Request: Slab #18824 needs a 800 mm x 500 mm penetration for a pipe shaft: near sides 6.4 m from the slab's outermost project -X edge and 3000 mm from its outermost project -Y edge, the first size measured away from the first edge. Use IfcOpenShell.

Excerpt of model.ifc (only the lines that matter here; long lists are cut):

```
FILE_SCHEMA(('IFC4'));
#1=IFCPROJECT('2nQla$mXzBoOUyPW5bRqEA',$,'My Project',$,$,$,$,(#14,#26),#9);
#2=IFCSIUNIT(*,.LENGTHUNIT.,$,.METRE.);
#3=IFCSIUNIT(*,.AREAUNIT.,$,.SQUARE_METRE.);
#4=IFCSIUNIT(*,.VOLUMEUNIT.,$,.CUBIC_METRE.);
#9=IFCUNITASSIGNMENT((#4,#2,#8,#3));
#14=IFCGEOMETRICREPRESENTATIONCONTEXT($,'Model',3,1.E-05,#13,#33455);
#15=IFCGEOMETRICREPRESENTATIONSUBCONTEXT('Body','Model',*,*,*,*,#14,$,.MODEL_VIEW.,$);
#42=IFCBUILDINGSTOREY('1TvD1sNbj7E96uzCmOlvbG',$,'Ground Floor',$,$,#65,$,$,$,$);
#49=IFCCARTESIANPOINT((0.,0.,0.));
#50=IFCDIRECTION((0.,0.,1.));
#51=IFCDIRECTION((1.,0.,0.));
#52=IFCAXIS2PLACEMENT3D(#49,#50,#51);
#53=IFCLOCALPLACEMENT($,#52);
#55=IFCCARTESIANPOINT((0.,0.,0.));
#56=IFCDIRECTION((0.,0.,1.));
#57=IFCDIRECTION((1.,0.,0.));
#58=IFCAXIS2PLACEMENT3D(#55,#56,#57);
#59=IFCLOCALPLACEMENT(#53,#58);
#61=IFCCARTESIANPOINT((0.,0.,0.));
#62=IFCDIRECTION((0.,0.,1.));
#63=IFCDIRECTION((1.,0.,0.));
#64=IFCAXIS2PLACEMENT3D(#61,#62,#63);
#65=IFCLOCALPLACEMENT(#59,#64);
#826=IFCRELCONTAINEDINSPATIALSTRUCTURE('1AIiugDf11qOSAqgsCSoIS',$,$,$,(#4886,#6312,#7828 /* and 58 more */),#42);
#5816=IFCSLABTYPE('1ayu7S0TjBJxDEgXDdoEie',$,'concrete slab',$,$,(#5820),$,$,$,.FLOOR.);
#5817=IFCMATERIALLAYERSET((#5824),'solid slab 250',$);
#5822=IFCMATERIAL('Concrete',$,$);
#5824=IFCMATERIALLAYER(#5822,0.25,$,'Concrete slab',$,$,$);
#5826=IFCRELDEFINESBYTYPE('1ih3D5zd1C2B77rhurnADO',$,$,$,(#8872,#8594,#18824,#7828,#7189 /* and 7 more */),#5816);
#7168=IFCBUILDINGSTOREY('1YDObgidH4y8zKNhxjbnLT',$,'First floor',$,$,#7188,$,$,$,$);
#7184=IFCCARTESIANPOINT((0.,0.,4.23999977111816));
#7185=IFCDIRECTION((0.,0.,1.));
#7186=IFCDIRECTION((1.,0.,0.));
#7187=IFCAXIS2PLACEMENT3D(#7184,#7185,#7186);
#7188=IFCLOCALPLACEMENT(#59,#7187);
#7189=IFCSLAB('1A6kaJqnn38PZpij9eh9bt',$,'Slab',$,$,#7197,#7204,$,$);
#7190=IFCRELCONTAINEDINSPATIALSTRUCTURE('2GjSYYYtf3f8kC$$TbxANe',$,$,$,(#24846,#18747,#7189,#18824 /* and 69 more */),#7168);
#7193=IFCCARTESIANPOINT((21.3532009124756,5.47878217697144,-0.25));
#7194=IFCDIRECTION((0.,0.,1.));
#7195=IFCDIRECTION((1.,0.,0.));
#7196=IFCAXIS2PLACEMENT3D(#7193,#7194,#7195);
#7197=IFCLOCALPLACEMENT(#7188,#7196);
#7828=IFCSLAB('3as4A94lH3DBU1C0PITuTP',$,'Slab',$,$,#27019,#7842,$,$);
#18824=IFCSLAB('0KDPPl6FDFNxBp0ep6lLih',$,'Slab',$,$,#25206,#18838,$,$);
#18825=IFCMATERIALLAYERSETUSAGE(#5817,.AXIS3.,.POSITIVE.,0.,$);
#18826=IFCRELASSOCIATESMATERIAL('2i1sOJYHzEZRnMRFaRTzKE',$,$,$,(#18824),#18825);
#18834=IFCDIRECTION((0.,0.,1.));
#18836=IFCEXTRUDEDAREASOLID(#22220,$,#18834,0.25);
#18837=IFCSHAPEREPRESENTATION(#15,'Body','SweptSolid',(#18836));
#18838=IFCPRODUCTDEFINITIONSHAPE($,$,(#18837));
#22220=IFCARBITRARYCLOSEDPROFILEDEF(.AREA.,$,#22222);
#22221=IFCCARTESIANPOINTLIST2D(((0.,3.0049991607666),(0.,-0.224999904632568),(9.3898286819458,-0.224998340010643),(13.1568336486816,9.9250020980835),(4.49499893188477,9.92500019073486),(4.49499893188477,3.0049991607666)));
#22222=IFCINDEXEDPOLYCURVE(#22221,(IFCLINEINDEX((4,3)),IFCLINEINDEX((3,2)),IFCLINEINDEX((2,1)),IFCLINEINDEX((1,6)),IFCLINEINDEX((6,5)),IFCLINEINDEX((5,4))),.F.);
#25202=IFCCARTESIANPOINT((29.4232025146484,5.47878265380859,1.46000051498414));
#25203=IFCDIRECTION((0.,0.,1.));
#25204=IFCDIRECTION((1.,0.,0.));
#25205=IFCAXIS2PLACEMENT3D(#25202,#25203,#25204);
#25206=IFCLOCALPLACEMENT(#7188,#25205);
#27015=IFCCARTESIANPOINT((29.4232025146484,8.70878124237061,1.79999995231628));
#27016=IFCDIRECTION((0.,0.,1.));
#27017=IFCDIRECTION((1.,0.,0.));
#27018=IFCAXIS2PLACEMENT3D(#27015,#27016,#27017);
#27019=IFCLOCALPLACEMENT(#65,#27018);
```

```python
import numpy as np
import ifcopenshell
import ifcopenshell.api.feature
import ifcopenshell.api.geometry
import ifcopenshell.api.root
import ifcopenshell.geom
import ifcopenshell.util.placement
import ifcopenshell.util.representation
import ifcopenshell.util.shape
import ifcopenshell.util.unit

model = ifcopenshell.open("model.ifc")
unit_scale = ifcopenshell.util.unit.calculate_unit_scale(model)
settings = ifcopenshell.geom.settings()


def volume(element):
    """Net volume in cubic metres, openings subtracted."""
    shape = ifcopenshell.geom.create_shape(settings, element)
    return ifcopenshell.util.shape.get_volume(shape.geometry)


slab = model.by_id(18824)
before = volume(slab)

# Extent in the slab's own axes, in metres. The edges named are its -X and -Y sides.
slab_shape = ifcopenshell.geom.create_shape(settings, slab)
vertices = ifcopenshell.util.shape.get_vertices(slab_shape.geometry)
x_min, y_min, bottom = vertices.min(axis=0)
top = vertices[:, 2].max()

opening = ifcopenshell.api.root.create_entity(model, ifc_class="IfcOpeningElement", name="Pipe shaft opening", predefined_type="OPENING")
context = ifcopenshell.util.representation.get_context(model, "Model", "Body", "MODEL_VIEW")
width, depth = 0.8, 0.5
outline = [(0.0, 0.0), (width, 0.0), (width, depth), (0.0, depth), (0.0, 0.0)]
# Overshoot both faces by 50 mm so the cut is clean.
shape = ifcopenshell.api.geometry.add_slab_representation(
    model, context=context, depth=top - bottom + 0.1, polyline=outline
)
ifcopenshell.api.geometry.assign_representation(model, product=opening, representation=shape)

matrix = ifcopenshell.util.placement.get_local_placement(slab.ObjectPlacement)
matrix[:, 3] = matrix @ np.append(np.array([x_min + 6.4, y_min + 3, bottom - 0.05]) / unit_scale, 1.0)
ifcopenshell.api.geometry.edit_object_placement(model, product=opening, matrix=matrix, is_si=False)
ifcopenshell.api.feature.add_feature(model, feature=opening, element=slab)

after = volume(slab)

print(f"slab volume {before:.3f} -> {after:.3f} m3")

model.write("model_edited.ifc")
```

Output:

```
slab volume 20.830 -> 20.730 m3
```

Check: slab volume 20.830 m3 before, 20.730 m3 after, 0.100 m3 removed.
